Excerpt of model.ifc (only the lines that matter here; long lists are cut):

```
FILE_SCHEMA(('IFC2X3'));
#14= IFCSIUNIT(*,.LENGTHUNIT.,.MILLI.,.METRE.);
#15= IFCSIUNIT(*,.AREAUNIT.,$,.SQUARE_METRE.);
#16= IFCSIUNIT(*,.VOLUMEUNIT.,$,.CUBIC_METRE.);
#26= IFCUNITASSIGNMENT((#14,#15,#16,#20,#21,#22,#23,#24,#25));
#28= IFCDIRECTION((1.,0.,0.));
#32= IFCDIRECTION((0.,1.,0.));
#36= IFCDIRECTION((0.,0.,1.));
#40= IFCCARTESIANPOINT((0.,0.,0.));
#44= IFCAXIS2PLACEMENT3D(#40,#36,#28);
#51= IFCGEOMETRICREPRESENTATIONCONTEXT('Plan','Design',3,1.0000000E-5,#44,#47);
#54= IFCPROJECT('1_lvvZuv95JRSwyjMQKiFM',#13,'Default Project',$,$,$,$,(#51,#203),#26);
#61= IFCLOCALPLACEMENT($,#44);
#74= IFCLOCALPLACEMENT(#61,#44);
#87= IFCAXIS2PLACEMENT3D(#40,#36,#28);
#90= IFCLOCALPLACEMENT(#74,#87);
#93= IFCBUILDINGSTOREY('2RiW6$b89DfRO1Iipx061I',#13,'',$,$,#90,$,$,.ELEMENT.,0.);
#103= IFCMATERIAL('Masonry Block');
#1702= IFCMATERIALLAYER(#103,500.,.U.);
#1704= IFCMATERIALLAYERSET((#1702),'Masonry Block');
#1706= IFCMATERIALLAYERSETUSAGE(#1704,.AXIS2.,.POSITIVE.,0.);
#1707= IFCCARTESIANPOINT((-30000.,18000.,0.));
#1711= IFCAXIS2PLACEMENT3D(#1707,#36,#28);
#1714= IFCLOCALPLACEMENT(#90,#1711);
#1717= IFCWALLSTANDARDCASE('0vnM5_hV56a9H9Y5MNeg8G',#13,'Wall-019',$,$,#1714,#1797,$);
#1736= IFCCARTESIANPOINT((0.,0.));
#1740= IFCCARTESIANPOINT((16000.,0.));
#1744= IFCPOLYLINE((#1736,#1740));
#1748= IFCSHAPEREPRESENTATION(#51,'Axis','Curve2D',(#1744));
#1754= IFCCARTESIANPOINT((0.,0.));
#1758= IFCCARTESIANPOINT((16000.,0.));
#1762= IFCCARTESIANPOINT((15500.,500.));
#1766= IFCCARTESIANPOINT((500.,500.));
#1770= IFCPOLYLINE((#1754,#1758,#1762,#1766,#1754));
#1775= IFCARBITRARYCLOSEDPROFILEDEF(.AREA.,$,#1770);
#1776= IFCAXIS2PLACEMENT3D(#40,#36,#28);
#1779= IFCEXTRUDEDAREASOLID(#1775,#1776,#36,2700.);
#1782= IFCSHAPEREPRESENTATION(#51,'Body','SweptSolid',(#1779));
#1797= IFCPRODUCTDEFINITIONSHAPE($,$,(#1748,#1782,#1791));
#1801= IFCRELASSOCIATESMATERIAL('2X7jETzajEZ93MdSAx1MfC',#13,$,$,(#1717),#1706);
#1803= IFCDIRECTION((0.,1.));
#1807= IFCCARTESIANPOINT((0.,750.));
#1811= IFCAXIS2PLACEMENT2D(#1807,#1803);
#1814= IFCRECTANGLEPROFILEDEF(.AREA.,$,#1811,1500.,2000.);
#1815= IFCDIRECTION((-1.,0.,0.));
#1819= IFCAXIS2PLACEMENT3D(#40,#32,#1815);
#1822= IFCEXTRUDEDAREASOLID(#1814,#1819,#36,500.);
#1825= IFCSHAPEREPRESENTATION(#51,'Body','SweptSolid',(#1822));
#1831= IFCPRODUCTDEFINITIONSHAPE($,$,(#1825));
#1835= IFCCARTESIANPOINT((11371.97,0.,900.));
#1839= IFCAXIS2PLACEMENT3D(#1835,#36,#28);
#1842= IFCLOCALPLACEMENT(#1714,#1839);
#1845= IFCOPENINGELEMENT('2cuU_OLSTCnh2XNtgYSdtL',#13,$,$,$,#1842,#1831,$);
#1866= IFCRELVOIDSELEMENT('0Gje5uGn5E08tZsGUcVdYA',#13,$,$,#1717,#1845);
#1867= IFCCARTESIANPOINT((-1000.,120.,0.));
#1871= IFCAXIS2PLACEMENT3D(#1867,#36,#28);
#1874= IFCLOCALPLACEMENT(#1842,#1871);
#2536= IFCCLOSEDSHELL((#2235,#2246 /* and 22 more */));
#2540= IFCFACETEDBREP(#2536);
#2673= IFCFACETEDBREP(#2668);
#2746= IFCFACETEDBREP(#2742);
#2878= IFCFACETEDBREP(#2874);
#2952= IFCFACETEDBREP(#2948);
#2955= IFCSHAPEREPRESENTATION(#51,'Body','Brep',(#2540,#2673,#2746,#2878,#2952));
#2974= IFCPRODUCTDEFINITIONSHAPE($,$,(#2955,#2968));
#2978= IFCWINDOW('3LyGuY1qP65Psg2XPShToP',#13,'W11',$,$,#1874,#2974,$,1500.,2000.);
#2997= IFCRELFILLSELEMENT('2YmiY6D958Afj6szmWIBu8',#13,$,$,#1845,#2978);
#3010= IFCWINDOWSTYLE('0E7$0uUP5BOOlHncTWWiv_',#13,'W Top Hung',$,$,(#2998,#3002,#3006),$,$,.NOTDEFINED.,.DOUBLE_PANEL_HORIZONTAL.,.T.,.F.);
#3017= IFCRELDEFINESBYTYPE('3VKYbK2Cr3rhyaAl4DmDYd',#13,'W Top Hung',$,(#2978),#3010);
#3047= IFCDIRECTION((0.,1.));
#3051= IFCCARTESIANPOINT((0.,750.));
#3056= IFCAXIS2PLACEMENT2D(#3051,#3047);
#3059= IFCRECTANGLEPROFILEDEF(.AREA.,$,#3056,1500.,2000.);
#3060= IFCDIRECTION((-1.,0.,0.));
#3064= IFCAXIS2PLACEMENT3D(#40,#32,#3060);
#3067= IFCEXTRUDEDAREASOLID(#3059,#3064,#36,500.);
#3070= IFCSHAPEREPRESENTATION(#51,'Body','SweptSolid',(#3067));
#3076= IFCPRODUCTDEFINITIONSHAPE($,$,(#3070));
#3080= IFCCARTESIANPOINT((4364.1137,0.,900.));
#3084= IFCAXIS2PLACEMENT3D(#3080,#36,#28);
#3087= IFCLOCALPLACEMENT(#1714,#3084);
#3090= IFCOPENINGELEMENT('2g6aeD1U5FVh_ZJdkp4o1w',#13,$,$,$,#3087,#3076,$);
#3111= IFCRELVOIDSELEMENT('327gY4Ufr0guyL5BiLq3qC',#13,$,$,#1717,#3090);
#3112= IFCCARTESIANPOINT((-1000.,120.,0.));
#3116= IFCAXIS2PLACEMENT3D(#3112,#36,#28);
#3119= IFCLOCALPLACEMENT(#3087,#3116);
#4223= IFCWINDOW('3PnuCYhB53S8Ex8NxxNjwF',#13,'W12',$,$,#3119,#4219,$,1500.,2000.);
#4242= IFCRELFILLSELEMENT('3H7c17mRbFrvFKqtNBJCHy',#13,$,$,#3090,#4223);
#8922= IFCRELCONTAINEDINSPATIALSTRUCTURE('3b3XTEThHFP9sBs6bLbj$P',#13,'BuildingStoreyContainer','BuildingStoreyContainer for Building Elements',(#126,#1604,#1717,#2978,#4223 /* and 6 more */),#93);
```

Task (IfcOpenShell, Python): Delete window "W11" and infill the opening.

```python
import ifcopenshell
import ifcopenshell.api.feature
import ifcopenshell.api.root
import ifcopenshell.geom
import ifcopenshell.util.shape

model = ifcopenshell.open("model.ifc")
settings = ifcopenshell.geom.settings()


def volume(element):
    """Net volume in cubic metres, openings subtracted."""
    shape = ifcopenshell.geom.create_shape(settings, element)
    return ifcopenshell.util.shape.get_volume(shape.geometry)


window = model.by_guid("3LyGuY1qP65Psg2XPShToP")
opening = window.FillsVoids[0].RelatingOpeningElement
wall = opening.VoidsElements[0].RelatingBuildingElement
before = volume(wall)

ifcopenshell.api.root.remove_product(model, product=window)
ifcopenshell.api.feature.remove_feature(model, feature=opening)

after = volume(wall)

print(f"wall volume {before:.3f} -> {after:.3f} m3")

model.write("model_updated.ifc")
```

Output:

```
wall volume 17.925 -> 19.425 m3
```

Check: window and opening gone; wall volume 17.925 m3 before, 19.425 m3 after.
